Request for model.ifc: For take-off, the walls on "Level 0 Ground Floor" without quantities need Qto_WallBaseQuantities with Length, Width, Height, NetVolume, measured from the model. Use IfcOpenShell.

First a look at what the model holds.

```python
import ifcopenshell
import ifcopenshell.util.element
import ifcopenshell.util.unit

model = ifcopenshell.open("model.ifc")
print(model.schema)
for unit_type in ("LENGTHUNIT", "AREAUNIT", "VOLUMEUNIT"):
    print(unit_type, ifcopenshell.util.unit.calculate_unit_scale(model, unit_type))
storey = next(s for s in model.by_type("IfcBuildingStorey") if s.Name == "Level 0 Ground Floor")
walls = [e for e in ifcopenshell.util.element.get_decomposition(storey) if e.is_a("IfcWall")]
for e in sorted(walls, key=lambda e: e.id()):
    print(e.id(), e.is_a(), e.Name, list(ifcopenshell.util.element.get_psets(e, qtos_only=True)), sep=" | ")
```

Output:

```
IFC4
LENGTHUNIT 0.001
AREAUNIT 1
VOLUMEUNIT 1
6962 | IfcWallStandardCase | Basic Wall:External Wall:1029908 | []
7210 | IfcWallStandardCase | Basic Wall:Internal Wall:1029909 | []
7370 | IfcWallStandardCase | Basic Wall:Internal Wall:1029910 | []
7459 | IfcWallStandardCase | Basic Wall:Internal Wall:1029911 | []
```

```python
import ifcopenshell
import ifcopenshell.api.pset
import ifcopenshell.geom
import ifcopenshell.util.element
import ifcopenshell.util.shape
import ifcopenshell.util.unit

model = ifcopenshell.open("model.ifc")
unit_scale = ifcopenshell.util.unit.calculate_unit_scale(model)
volume_scale = ifcopenshell.util.unit.calculate_unit_scale(model, "VOLUMEUNIT")
settings = ifcopenshell.geom.settings()

storey = next(s for s in model.by_type("IfcBuildingStorey") if s.Name == "Level 0 Ground Floor")
walls = [e for e in ifcopenshell.util.element.get_decomposition(storey) if e.is_a("IfcWall")]

for e in sorted(walls, key=lambda e: e.id()):
    if ifcopenshell.util.element.get_psets(e, qtos_only=True, should_inherit=False):
        continue
    # Geometry comes back in metres, in the element's own axes.
    shape = ifcopenshell.geom.create_shape(settings, e)
    values = {
        "Length": ifcopenshell.util.shape.get_x(shape.geometry) / unit_scale,
        "Width": ifcopenshell.util.shape.get_y(shape.geometry) / unit_scale,
        "Height": ifcopenshell.util.shape.get_z(shape.geometry) / unit_scale,
        "NetVolume": ifcopenshell.util.shape.get_volume(shape.geometry) / volume_scale,
    }
    qto = ifcopenshell.api.pset.add_qto(model, product=e, name="Qto_WallBaseQuantities")
    ifcopenshell.api.pset.edit_qto(model, qto=qto, properties=values)
    print(e.id(), {k: round(v, 3) for k, v in values.items()})

model.write("model-out.ifc")
```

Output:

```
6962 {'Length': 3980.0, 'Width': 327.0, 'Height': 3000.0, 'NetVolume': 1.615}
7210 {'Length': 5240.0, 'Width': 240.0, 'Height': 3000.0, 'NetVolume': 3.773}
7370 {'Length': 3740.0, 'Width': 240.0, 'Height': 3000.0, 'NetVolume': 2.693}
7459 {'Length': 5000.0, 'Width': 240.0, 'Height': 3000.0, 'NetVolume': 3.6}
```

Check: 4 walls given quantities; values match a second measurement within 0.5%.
